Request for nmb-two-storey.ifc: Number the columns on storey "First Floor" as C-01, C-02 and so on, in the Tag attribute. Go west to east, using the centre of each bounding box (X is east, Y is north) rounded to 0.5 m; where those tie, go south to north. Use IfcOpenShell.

First a look at what the model holds.

```python
import ifcopenshell
import ifcopenshell.util.element
import ifcopenshell.util.placement

model = ifcopenshell.open("nmb-two-storey.ifc")
print(model.schema)
storey = next(s for s in model.by_type("IfcBuildingStorey") if s.Name == "First Floor")
columns = [e for e in ifcopenshell.util.element.get_decomposition(storey) if e.is_a("IfcColumn")]
for e in sorted(columns, key=lambda e: e.id()):
    origin = ifcopenshell.util.placement.get_local_placement(e.ObjectPlacement)[:3, 3]
    print(e.id(), e.Tag, e.Name, origin.round(2) + 0.0, sep=" | ")
```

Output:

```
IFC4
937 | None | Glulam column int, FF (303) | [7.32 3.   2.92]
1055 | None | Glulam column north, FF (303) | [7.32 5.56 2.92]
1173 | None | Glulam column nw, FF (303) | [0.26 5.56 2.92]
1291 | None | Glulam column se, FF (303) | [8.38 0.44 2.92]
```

```python
import ifcopenshell
import ifcopenshell.geom
import ifcopenshell.util.element
import ifcopenshell.util.shape

model = ifcopenshell.open("nmb-two-storey.ifc")
settings = ifcopenshell.geom.settings()
settings.set("use-world-coords", True)


def centre(element):
    shape = ifcopenshell.geom.create_shape(settings, element)
    return ifcopenshell.util.shape.get_bbox_centroid(shape.geometry)


storey = next(s for s in model.by_type("IfcBuildingStorey") if s.Name == "First Floor")
columns = [e for e in ifcopenshell.util.element.get_decomposition(storey) if e.is_a("IfcColumn")]

# Insertion points can sit at a corner or the storey origin, so sort by the geometry (in metres).
centres = {e: centre(e) for e in columns}
columns.sort(key=lambda e: (round(centres[e][0] / 0.5), centres[e][1]))

for i, e in enumerate(columns, start=1):
    number = f"C-{i:02d}"
    e.Tag = number
    print(e.id(), number)

model.write("nmb-two-storey_updated.ifc")
```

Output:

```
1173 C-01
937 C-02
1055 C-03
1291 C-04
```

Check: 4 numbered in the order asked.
